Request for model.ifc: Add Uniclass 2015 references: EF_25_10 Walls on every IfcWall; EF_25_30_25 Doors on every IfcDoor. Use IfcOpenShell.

First a look at what the model holds.

```python
import ifcopenshell

model = ifcopenshell.open("model.ifc")
print(model.schema)
print("classifications:", [c.Name for c in model.by_type("IfcClassification")])
for ifc_class in ("IfcDoor", "IfcRoof", "IfcStair", "IfcWall", "IfcWindow"):
    print(ifc_class, len(model.by_type(ifc_class)))
```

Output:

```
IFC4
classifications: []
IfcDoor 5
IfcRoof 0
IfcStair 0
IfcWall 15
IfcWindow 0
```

```python
import ifcopenshell
import ifcopenshell.api.classification

model = ifcopenshell.open("model.ifc")

system = ifcopenshell.api.classification.add_classification(model, classification="Uniclass 2015")

codes = {
    "IfcWall": ("EF_25_10", "Walls"),
    "IfcDoor": ("EF_25_30_25", "Doors"),
}
for ifc_class, (code, name) in codes.items():
    products = model.by_type(ifc_class)
    ifcopenshell.api.classification.add_reference(
        model, products=products, classification=system, identification=code, name=name
    )
    print(code, len(products))

model.write("model_edited.ifc")
```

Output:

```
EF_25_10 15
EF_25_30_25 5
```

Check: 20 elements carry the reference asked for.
